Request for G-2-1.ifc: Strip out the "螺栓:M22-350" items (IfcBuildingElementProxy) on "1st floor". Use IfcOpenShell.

First a look at what the model holds.

```python
import ifcopenshell
import ifcopenshell.util.element

model = ifcopenshell.open("G-2-1.ifc")
print(model.schema)
storey = next(s for s in model.by_type("IfcBuildingStorey") if s.Name == "1st floor")
proxies = [e for e in ifcopenshell.util.element.get_decomposition(storey) if e.is_a("IfcBuildingElementProxy")]
seen = {}
for e in proxies:
    element_type = ifcopenshell.util.element.get_type(e)
    name = element_type.Name if element_type not in (None, e) else None
    seen[name] = seen.get(name, 0) + 1
for name, count in sorted(seen.items(), key=str):
    print(count, "x", name)
```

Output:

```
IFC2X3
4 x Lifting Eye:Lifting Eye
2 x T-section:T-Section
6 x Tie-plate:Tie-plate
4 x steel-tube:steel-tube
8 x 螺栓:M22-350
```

```python
import ifcopenshell
import ifcopenshell.api.root
import ifcopenshell.util.element

model = ifcopenshell.open("G-2-1.ifc")

storey = next(s for s in model.by_type("IfcBuildingStorey") if s.Name == "1st floor")
proxies = [e for e in ifcopenshell.util.element.get_decomposition(storey) if e.is_a("IfcBuildingElementProxy")]
targets = [e for e in proxies if (t := ifcopenshell.util.element.get_type(e)) not in (None, e) and t.Name == "螺栓:M22-350"]

for e in targets:
    ifcopenshell.api.root.remove_product(model, product=e)
print(len(targets), "removed")

model.write("G-2-1_updated.ifc")
```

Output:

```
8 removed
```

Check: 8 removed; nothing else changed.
